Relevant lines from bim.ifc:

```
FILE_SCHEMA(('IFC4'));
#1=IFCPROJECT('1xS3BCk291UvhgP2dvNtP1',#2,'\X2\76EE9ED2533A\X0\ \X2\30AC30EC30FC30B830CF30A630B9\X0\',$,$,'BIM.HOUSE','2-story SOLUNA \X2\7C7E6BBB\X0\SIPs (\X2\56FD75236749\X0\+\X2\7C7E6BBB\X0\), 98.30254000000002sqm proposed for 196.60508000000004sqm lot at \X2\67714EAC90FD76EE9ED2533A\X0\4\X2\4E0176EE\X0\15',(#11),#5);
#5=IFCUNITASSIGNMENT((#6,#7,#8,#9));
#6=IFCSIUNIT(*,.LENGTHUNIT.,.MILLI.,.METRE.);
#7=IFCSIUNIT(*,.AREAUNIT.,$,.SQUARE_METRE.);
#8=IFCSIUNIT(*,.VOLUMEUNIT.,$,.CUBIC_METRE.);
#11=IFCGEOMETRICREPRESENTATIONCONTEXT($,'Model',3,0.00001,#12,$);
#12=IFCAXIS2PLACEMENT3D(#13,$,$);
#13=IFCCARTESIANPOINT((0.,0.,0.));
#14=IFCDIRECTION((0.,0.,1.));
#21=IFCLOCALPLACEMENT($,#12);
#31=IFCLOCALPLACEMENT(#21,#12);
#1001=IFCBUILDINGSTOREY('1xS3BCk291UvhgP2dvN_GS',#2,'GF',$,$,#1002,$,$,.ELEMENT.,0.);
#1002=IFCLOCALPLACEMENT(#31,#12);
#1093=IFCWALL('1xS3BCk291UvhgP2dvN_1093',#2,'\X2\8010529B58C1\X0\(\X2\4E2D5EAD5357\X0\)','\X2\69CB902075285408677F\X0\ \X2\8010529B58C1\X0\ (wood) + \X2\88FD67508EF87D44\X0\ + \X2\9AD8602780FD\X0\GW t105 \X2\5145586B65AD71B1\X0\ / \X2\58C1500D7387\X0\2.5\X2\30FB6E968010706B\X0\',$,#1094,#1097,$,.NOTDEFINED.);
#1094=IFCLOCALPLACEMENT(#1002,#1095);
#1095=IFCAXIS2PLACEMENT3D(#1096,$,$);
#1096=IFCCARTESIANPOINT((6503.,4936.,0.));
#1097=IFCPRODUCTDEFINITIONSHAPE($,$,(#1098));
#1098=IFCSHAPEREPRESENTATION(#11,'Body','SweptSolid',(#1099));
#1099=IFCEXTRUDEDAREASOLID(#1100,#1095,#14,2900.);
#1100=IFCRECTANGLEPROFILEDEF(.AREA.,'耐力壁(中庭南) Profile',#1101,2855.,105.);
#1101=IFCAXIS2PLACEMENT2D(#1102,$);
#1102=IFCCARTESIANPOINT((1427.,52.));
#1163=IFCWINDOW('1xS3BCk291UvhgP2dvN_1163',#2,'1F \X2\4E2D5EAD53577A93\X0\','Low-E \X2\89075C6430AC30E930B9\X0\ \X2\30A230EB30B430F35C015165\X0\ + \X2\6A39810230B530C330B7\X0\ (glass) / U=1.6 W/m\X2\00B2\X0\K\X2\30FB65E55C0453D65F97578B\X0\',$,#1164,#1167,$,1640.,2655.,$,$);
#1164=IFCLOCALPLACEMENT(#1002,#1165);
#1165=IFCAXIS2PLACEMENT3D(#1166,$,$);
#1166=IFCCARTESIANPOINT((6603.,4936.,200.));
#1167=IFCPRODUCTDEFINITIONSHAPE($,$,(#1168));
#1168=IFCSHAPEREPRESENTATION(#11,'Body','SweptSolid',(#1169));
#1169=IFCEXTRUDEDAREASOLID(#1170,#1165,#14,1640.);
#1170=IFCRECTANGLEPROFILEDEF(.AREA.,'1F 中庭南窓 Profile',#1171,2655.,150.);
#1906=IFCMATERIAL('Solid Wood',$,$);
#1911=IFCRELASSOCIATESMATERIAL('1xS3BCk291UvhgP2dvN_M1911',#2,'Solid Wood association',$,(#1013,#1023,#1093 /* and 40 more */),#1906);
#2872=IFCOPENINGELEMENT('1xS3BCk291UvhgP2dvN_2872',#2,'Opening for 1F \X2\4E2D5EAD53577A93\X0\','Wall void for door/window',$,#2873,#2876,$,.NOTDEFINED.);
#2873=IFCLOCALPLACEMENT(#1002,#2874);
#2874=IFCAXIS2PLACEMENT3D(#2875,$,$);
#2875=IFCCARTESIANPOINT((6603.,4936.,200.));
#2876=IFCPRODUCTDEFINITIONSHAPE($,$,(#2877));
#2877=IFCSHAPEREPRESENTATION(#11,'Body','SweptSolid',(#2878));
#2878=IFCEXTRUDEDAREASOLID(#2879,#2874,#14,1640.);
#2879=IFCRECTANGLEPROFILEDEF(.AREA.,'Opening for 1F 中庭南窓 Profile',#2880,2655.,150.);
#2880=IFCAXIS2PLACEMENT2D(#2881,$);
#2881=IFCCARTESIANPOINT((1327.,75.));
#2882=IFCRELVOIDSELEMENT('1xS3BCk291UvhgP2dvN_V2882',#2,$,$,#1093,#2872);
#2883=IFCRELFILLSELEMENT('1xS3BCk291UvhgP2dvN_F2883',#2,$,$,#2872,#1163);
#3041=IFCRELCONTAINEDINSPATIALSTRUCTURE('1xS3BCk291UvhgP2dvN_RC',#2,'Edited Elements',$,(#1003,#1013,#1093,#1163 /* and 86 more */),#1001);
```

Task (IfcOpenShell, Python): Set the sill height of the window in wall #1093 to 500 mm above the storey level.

```python
import numpy as np
import ifcopenshell
import ifcopenshell.api.geometry
import ifcopenshell.geom
import ifcopenshell.util.element
import ifcopenshell.util.placement
import ifcopenshell.util.shape
import ifcopenshell.util.unit

model = ifcopenshell.open("bim.ifc")
unit_scale = ifcopenshell.util.unit.calculate_unit_scale(model)

window = model.by_guid("1xS3BCk291UvhgP2dvN_1163")
opening = window.FillsVoids[0].RelatingOpeningElement
storey = ifcopenshell.util.element.get_container(window, ifc_class="IfcBuildingStorey")
level = ifcopenshell.util.placement.get_local_placement(storey.ObjectPlacement)[2, 3]

# The opening's origin need not be at the sill, so measure its lowest point.
shape = ifcopenshell.geom.create_shape(ifcopenshell.geom.settings(), opening)
bottom = ifcopenshell.util.shape.get_shape_bottom_elevation(shape, shape.geometry) / unit_scale
dz = level + 0.5 / unit_scale - bottom

shift = np.array([0.0, 0.0, dz])
# The window is not placed relative to its opening, so move both.
for product in (opening, window):
    matrix = ifcopenshell.util.placement.get_local_placement(product.ObjectPlacement)
    matrix[:3, 3] += shift
    ifcopenshell.api.geometry.edit_object_placement(model, product=product, matrix=matrix, is_si=False)

print(f"moved by {dz * unit_scale:+.3f} m")

model.write("bim-out.ifc")
```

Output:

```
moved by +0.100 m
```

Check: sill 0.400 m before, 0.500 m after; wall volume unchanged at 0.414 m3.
